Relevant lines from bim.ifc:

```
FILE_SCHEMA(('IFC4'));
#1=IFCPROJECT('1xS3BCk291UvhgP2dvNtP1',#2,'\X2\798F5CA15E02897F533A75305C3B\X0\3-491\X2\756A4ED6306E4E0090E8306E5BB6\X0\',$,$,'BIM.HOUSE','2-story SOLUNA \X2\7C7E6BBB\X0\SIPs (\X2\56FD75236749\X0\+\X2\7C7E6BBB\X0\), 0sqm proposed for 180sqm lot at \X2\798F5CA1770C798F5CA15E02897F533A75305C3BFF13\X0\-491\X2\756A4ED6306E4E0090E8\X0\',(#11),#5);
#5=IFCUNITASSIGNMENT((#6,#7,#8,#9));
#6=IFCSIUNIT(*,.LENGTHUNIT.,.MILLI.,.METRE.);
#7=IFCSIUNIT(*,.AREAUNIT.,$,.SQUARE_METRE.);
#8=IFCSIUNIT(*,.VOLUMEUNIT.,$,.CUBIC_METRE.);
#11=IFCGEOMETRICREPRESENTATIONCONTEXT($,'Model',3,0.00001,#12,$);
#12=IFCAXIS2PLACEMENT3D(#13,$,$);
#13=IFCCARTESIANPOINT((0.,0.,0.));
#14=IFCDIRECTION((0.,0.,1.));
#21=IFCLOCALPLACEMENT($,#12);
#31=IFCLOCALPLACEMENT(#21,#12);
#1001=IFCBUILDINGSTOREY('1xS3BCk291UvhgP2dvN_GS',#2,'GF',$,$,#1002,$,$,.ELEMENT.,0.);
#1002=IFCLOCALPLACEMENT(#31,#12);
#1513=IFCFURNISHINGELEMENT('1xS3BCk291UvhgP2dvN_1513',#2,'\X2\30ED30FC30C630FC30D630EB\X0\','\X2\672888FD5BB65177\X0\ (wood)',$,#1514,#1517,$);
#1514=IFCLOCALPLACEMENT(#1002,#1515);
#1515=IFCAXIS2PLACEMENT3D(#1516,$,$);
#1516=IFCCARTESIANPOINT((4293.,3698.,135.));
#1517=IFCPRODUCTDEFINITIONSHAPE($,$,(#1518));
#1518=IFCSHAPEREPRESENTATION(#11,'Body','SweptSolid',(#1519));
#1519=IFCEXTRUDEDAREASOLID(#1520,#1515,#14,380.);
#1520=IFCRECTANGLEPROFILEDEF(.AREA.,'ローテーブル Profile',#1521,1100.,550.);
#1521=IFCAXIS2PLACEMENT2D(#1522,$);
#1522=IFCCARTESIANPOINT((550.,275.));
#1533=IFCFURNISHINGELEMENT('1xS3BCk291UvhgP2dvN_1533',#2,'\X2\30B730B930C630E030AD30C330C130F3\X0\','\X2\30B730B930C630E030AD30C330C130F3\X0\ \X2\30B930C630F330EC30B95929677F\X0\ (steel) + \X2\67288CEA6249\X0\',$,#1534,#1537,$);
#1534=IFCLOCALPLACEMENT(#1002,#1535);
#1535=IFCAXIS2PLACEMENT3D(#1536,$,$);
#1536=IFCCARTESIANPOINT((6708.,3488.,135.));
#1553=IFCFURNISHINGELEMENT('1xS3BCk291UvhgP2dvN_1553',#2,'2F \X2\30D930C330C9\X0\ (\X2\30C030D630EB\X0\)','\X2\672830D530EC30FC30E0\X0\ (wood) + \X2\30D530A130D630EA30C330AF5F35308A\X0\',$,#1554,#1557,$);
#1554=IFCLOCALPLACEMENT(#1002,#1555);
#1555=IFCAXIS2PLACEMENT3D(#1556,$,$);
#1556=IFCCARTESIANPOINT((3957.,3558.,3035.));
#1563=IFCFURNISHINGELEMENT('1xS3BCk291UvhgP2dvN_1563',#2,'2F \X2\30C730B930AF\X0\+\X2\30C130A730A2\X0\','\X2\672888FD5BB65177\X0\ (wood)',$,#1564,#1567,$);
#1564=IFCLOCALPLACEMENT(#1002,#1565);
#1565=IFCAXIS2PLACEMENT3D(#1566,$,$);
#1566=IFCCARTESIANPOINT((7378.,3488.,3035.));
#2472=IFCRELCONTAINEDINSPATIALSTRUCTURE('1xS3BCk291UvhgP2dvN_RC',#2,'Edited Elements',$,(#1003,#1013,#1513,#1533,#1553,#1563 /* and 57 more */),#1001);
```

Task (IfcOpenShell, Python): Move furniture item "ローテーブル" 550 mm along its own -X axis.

```python
import ifcopenshell
import ifcopenshell.api.geometry
import ifcopenshell.util.placement

model = ifcopenshell.open("bim.ifc")

item = model.by_guid("1xS3BCk291UvhgP2dvN_1513")
matrix = ifcopenshell.util.placement.get_local_placement(item.ObjectPlacement)
matrix[:3, 3] -= matrix[:3, 0] * 550.0
ifcopenshell.api.geometry.edit_object_placement(model, product=item, matrix=matrix, is_si=False)

print(ifcopenshell.util.placement.get_local_placement(item.ObjectPlacement).round(3) + 0.0)

model.write("bim_edited.ifc")
```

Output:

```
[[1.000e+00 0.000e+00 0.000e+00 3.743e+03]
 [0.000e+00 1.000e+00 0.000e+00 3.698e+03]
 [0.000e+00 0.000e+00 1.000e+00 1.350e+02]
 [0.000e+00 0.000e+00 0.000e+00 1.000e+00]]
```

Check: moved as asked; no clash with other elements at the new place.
